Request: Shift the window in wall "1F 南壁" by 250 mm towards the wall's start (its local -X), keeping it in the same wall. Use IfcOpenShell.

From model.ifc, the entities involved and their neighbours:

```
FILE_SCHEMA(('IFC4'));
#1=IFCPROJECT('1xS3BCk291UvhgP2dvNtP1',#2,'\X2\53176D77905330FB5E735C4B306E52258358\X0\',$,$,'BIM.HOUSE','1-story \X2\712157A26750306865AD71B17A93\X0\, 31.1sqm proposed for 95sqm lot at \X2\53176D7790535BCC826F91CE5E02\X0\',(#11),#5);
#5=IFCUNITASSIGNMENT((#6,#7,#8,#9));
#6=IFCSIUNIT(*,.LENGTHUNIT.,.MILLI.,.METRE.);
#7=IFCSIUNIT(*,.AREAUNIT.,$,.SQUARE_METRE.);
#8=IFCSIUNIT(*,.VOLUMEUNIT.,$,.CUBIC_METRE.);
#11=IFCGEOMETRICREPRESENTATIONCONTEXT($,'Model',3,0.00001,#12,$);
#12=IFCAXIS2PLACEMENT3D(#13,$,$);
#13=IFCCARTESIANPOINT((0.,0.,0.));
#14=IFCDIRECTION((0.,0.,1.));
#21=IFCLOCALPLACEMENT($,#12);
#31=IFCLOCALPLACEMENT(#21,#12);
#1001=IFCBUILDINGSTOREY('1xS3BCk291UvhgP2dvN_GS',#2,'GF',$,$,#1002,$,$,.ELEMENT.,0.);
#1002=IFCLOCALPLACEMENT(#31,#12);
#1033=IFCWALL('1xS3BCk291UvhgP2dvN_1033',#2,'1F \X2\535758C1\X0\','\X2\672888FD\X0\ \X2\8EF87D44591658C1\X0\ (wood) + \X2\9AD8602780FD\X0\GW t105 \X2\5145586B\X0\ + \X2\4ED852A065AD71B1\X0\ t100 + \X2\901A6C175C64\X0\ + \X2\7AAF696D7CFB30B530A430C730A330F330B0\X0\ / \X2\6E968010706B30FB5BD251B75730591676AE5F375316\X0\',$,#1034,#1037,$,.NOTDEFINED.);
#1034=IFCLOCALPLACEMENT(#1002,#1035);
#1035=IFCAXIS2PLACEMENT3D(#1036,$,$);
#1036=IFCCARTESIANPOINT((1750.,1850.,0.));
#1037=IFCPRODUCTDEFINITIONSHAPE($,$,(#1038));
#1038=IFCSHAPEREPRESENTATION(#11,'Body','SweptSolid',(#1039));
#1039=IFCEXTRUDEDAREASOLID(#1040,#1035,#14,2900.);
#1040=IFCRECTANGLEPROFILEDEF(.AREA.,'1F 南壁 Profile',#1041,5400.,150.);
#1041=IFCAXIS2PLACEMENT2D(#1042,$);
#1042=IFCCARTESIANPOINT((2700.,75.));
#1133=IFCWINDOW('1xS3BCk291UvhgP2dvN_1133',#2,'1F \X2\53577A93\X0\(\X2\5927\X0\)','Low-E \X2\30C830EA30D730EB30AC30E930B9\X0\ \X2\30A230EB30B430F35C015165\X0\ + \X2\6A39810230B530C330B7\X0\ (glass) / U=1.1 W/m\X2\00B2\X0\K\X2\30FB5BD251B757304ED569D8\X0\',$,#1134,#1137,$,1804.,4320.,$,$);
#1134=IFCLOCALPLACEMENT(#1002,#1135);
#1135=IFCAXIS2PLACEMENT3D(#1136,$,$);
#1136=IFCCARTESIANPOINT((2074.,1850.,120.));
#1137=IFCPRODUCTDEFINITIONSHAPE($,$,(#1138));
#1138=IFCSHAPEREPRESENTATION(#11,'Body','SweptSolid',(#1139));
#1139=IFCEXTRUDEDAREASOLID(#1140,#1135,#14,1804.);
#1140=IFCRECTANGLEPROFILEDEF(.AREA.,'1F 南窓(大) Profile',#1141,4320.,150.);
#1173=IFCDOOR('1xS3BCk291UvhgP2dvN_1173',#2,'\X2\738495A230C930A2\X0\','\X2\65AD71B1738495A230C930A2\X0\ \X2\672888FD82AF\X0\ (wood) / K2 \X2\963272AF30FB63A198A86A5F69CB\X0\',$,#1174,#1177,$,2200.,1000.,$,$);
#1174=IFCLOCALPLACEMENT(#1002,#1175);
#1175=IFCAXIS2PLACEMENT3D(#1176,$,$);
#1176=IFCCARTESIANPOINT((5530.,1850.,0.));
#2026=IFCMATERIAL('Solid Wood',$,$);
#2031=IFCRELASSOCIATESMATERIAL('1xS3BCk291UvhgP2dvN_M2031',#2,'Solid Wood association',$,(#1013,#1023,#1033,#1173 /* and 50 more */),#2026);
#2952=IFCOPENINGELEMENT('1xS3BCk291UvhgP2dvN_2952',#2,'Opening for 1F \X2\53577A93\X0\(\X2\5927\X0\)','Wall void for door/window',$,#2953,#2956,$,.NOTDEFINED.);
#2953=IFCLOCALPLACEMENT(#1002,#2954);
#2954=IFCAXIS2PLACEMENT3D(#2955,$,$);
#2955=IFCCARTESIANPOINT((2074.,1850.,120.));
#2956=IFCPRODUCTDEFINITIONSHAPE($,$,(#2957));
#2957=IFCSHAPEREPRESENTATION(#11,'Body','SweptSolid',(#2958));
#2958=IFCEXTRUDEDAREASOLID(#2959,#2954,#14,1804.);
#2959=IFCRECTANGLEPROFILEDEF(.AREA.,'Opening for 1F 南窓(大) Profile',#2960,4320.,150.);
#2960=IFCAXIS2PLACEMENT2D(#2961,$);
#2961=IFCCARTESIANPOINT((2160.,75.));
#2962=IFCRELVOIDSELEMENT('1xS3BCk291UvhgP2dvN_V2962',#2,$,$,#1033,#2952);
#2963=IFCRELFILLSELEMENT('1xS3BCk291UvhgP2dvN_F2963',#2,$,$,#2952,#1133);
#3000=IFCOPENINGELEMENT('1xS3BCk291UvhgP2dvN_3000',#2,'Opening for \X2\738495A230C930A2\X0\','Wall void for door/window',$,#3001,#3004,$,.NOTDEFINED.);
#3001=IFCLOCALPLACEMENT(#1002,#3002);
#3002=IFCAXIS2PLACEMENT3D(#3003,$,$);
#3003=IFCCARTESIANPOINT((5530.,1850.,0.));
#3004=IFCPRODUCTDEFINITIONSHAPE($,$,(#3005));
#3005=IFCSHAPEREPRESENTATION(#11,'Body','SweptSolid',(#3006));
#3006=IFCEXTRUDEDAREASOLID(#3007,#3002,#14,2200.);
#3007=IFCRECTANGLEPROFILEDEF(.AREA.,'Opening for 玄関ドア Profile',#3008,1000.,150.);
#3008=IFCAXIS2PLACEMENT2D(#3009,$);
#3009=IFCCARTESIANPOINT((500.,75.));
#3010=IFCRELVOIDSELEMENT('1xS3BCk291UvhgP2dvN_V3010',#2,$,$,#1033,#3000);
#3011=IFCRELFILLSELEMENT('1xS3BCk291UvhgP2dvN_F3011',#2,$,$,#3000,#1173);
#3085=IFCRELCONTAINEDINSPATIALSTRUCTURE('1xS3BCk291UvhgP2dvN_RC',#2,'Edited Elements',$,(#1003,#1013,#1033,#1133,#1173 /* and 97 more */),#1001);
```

```python
import ifcopenshell
import ifcopenshell.api.geometry
import ifcopenshell.util.placement
import ifcopenshell.util.unit

model = ifcopenshell.open("model.ifc")
unit_scale = ifcopenshell.util.unit.calculate_unit_scale(model)

window = model.by_id(1133)
opening = window.FillsVoids[0].RelatingOpeningElement
wall = opening.VoidsElements[0].RelatingBuildingElement

wall_matrix = ifcopenshell.util.placement.get_local_placement(wall.ObjectPlacement)
shift = wall_matrix[:3, 0] * -0.25 / unit_scale
before = ifcopenshell.util.placement.get_local_placement(window.ObjectPlacement)[:3, 3].copy()

# The window is not placed relative to its opening, so move both.
for product in (opening, window):
    matrix = ifcopenshell.util.placement.get_local_placement(product.ObjectPlacement)
    matrix[:3, 3] += shift
    ifcopenshell.api.geometry.edit_object_placement(model, product=product, matrix=matrix, is_si=False)

after = ifcopenshell.util.placement.get_local_placement(window.ObjectPlacement)[:3, 3]
print("window moved by", (after - before).round(3) + 0.0)

model.write("model_rev.ifc")
```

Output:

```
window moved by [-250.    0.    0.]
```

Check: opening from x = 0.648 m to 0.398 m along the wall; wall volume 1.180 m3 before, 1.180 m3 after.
